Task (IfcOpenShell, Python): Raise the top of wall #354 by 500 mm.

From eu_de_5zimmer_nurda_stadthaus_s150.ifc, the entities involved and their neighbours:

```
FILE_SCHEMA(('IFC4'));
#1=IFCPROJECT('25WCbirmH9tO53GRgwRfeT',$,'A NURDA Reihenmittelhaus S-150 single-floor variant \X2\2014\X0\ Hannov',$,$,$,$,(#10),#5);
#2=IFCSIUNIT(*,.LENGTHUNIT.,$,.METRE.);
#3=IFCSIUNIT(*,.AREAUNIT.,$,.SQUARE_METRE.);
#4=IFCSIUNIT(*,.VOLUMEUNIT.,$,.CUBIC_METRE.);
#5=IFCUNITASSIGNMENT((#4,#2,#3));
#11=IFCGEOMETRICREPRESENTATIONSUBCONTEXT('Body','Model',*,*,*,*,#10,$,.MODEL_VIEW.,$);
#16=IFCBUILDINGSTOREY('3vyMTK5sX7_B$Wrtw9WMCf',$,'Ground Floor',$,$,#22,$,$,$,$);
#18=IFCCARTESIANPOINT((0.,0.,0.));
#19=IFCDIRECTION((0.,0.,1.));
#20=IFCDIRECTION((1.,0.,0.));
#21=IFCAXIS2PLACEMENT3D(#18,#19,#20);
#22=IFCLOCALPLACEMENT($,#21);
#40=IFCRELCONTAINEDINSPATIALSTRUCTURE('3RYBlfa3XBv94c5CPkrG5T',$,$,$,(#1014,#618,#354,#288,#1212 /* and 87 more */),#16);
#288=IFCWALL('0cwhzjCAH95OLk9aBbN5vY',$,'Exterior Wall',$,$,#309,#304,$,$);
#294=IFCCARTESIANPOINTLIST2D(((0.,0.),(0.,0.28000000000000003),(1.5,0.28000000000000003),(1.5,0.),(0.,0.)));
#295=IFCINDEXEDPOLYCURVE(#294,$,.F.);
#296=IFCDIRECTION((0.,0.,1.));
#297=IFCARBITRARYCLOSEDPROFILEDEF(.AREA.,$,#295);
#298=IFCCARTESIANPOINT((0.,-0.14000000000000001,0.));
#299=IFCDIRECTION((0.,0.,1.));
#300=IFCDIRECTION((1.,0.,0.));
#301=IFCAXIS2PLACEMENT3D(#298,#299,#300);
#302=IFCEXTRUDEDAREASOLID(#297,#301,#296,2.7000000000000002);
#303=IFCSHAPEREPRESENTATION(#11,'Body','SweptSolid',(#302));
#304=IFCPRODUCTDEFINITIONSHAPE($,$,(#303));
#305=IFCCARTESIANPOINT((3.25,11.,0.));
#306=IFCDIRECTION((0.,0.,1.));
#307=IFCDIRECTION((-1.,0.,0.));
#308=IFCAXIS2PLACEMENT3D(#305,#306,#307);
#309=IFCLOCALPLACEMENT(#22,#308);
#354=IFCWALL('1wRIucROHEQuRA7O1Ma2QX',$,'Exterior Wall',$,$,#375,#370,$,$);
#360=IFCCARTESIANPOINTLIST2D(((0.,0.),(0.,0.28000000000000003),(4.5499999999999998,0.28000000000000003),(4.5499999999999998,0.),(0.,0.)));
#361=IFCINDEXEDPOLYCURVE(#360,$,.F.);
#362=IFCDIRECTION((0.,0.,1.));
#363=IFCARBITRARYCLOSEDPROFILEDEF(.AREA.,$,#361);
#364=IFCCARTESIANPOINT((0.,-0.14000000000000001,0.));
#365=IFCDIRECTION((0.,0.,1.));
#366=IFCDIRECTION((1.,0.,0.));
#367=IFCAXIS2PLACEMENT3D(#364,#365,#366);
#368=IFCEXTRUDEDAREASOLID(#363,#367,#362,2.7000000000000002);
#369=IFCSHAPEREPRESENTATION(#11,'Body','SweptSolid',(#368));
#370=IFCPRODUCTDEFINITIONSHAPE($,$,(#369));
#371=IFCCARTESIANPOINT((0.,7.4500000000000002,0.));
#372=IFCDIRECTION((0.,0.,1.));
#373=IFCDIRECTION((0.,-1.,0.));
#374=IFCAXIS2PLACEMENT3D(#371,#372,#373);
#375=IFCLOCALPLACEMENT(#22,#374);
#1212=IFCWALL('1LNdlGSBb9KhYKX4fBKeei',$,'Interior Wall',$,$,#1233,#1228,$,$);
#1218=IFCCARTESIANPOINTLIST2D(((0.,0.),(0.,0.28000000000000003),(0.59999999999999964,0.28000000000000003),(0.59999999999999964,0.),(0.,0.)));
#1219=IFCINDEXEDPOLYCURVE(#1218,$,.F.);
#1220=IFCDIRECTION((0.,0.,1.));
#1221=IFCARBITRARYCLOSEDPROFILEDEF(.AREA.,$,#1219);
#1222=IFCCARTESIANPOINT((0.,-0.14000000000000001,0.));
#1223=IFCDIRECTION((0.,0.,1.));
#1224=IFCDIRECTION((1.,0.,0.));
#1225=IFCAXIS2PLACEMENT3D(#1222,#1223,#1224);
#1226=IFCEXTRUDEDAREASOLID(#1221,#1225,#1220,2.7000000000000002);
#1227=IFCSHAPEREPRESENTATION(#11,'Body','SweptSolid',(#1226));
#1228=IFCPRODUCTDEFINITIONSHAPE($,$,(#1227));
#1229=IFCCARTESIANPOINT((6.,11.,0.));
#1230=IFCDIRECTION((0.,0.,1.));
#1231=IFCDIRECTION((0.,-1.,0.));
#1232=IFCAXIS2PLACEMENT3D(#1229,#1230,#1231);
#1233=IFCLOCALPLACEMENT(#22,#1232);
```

```python
import ifcopenshell
import ifcopenshell.geom
import ifcopenshell.util.representation
import ifcopenshell.util.shape

model = ifcopenshell.open("eu_de_5zimmer_nurda_stadthaus_s150.ifc")
settings = ifcopenshell.geom.settings()


def volume(element):
    """Net volume in cubic metres, openings subtracted."""
    shape = ifcopenshell.geom.create_shape(settings, element)
    return ifcopenshell.util.shape.get_volume(shape.geometry)


wall = model.by_guid("1wRIucROHEQuRA7O1Ma2QX")
before = volume(wall)

body = ifcopenshell.util.representation.get_representation(wall, "Model", "Body")
solid = body.Items[0]
old_height = solid.Depth
solid.Depth += 0.5
after = volume(wall)

print(f"height {old_height:g} -> {solid.Depth:g}, volume {before:.3f} -> {after:.3f} m3")

model.write("eu_de_5zimmer_nurda_stadthaus_s150_rev.ifc")
```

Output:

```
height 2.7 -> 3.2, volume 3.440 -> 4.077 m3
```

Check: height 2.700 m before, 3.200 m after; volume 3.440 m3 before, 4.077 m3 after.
